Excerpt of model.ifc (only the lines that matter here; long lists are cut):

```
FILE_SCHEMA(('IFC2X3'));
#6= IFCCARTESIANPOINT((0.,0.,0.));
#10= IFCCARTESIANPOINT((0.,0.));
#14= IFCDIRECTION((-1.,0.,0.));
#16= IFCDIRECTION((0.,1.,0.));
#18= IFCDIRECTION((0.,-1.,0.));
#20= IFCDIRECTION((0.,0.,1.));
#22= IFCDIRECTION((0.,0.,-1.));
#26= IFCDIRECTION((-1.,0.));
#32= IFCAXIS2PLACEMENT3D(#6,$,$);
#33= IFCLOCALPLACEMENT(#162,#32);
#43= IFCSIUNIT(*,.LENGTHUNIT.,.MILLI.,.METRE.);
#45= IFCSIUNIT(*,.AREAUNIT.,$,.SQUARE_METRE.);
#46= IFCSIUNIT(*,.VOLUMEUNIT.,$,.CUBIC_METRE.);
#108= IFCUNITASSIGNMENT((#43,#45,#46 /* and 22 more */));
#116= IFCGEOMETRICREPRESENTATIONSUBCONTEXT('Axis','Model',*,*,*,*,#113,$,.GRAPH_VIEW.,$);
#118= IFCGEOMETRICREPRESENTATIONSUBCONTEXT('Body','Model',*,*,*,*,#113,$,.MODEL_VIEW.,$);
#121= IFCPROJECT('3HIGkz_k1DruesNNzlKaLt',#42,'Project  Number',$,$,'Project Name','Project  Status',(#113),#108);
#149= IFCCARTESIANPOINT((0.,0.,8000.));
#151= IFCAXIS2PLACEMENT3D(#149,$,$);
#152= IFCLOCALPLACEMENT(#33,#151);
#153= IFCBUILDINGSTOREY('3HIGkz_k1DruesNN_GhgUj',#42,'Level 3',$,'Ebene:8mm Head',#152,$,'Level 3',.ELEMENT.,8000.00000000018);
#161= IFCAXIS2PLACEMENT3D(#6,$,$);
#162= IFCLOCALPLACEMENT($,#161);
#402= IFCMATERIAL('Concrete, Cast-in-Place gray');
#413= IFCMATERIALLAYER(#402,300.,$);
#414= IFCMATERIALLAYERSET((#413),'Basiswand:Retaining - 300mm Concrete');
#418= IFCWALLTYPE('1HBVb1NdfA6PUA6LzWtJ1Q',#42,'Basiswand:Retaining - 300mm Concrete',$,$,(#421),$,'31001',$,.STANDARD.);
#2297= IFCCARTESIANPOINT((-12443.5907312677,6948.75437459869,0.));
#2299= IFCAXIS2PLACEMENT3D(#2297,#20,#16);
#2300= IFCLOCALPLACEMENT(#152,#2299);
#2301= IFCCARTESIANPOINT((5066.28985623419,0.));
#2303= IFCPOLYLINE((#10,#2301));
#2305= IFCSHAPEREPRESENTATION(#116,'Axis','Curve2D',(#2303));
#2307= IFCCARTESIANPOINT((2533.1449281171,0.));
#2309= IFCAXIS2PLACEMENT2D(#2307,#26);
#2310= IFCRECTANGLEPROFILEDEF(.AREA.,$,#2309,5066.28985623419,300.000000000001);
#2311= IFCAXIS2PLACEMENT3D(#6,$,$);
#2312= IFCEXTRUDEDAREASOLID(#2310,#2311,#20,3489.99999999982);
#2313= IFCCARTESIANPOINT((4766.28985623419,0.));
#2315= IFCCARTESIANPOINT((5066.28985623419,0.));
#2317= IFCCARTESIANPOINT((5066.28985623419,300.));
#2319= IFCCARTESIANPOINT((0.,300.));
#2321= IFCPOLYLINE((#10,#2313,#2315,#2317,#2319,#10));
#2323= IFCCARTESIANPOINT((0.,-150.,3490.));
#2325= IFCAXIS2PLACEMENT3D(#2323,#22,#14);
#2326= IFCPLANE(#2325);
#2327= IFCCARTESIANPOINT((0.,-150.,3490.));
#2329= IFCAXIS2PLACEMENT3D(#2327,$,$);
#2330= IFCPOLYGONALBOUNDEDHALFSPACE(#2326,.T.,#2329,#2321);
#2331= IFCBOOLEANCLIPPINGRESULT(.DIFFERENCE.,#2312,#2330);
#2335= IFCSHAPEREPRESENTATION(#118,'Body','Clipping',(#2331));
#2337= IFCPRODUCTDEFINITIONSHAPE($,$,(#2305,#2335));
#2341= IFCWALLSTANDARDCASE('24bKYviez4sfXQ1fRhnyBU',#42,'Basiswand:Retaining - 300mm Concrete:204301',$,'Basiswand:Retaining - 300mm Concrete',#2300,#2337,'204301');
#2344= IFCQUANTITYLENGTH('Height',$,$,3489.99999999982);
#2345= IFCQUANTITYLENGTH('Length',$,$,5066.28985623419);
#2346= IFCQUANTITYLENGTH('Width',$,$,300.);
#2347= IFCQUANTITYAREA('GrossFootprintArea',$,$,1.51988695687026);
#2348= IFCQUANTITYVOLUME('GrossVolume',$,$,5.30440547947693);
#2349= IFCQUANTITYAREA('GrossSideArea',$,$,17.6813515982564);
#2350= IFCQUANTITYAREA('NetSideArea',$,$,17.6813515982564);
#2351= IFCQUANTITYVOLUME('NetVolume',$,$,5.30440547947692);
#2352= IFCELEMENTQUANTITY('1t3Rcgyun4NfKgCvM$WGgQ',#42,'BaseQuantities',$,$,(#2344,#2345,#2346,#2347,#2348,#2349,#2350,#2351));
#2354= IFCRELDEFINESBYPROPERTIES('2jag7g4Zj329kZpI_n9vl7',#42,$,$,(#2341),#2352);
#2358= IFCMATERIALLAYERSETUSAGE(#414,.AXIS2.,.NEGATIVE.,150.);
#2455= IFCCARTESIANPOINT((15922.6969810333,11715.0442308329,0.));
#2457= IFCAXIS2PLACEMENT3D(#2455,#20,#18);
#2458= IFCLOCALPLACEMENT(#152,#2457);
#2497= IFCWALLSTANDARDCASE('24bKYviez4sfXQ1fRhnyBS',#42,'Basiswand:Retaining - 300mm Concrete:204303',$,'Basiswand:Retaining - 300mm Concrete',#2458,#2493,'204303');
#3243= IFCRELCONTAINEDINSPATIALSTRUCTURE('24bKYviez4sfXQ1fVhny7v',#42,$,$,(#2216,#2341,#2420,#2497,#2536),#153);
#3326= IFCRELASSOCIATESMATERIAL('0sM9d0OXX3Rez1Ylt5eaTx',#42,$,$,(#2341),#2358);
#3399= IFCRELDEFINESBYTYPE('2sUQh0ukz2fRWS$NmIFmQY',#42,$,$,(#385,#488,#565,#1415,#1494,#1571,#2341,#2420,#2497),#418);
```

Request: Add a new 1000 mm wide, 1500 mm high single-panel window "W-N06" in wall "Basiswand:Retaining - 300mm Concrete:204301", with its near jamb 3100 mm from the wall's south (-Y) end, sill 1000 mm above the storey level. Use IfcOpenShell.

```python
import numpy as np
import ifcopenshell
import ifcopenshell.api.feature
import ifcopenshell.api.geometry
import ifcopenshell.api.pset
import ifcopenshell.api.root
import ifcopenshell.api.spatial
import ifcopenshell.api.type
import ifcopenshell.geom
import ifcopenshell.util.element
import ifcopenshell.util.placement
import ifcopenshell.util.representation
import ifcopenshell.util.shape
import ifcopenshell.util.unit

model = ifcopenshell.open("model.ifc")
unit_scale = ifcopenshell.util.unit.calculate_unit_scale(model)
area_scale = ifcopenshell.util.unit.calculate_unit_scale(model, "AREAUNIT")
volume_scale = ifcopenshell.util.unit.calculate_unit_scale(model, "VOLUMEUNIT")
settings = ifcopenshell.geom.settings()


def volume(element):
    """Net volume in cubic metres, openings subtracted."""
    shape = ifcopenshell.geom.create_shape(settings, element)
    return ifcopenshell.util.shape.get_volume(shape.geometry)


wall = model.by_id(2341)
storey = ifcopenshell.util.element.get_container(wall, ifc_class="IfcBuildingStorey")
context = ifcopenshell.util.representation.get_context(model, "Model", "Body", "MODEL_VIEW")
before = volume(wall)

width, height, from_end, sill = 1, 1.5, 3.1, 1  # metres

# The wall runs along its own X axis, and the end named is its -X end.
wall_shape = ifcopenshell.geom.create_shape(settings, wall)
x, y, z = ifcopenshell.util.shape.get_vertices(wall_shape.geometry).T
start = x.min() + from_end
face, thickness = float(y.min()), float(y.max() - y.min())
wall_matrix = ifcopenshell.util.placement.get_local_placement(wall.ObjectPlacement)
level = ifcopenshell.util.placement.get_local_placement(storey.ObjectPlacement)[2, 3]


def in_wall(x, y):
    """Placement at x, y metres in the wall's axes, at sill height."""
    matrix = wall_matrix.copy()
    matrix[:, 3] = wall_matrix @ np.array([x / unit_scale, y / unit_scale, 0.0, 1.0])
    matrix[2, 3] = level + sill / unit_scale
    return matrix


# Opening: a box that overshoots both wall faces by 50 mm.
opening = ifcopenshell.api.root.create_entity(model, ifc_class="IfcOpeningElement")
box = ifcopenshell.api.geometry.add_wall_representation(
    model, context=context, length=width, height=height, thickness=thickness + 0.1
)
ifcopenshell.api.geometry.assign_representation(model, product=opening, representation=box)
ifcopenshell.api.geometry.edit_object_placement(model, product=opening, matrix=in_wall(start, face - 0.05), is_si=False)
ifcopenshell.api.feature.add_feature(model, feature=opening, element=wall)

window = ifcopenshell.api.root.create_entity(model, ifc_class="IfcWindow", name="W-N06")
window.OverallWidth, window.OverallHeight = width / unit_scale, height / unit_scale
body = ifcopenshell.api.geometry.add_window_representation(
    model,
    context=context,
    overall_width=window.OverallWidth,
    overall_height=window.OverallHeight,
    partition_type="SINGLE_PANEL",
)
ifcopenshell.api.geometry.assign_representation(model, product=window, representation=body)
ifcopenshell.api.spatial.assign_container(model, products=[window], relating_structure=storey)
fills = ifcopenshell.api.feature.add_filling(model, opening=opening, element=window)
fills.OwnerHistory = window.OwnerHistory  # required in IFC2X3

# IFC2X3 keeps the operation on the window style.
style = ifcopenshell.api.root.create_entity(model, ifc_class="IfcWindowStyle", name="W-N06")
style.OperationType, style.ConstructionType = "SINGLE_PANEL", "NOTDEFINED"
style.ParameterTakesPrecedence = style.Sizeable = False
ifcopenshell.api.type.assign_type(model, related_objects=[window], relating_type=style)

# Centre the window in the wall's thickness.
ifcopenshell.api.geometry.edit_object_placement(model, product=window, matrix=in_wall(start, face), is_si=False)
window_shape = ifcopenshell.geom.create_shape(settings, window)
depth = ifcopenshell.util.shape.get_vertices(window_shape.geometry)[:, 1]
offset = face + thickness / 2 - (depth.min() + depth.max()) / 2
ifcopenshell.api.geometry.edit_object_placement(model, product=window, matrix=in_wall(start, offset), is_si=False)

after = volume(wall)

# Update the wall's stored quantities.
qto = model.by_id(ifcopenshell.util.element.get_pset(wall, "BaseQuantities", should_inherit=False)["id"])
ifcopenshell.api.pset.edit_qto(model, qto=qto, properties={
    "NetSideArea": after / thickness / area_scale,
    "NetVolume": after / volume_scale,
})

print(f"wall volume {before:.3f} -> {after:.3f} m3")

model.write("model-out.ifc")
```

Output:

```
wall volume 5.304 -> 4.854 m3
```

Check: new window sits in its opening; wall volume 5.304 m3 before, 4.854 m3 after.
